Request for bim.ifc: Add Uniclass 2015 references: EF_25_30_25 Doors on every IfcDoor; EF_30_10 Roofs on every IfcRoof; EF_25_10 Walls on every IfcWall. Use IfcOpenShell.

First a look at what the model holds.

```python
import ifcopenshell

model = ifcopenshell.open("bim.ifc")
print(model.schema)
print("classifications:", [c.Name for c in model.by_type("IfcClassification")])
for ifc_class in ("IfcDoor", "IfcRoof", "IfcStair", "IfcWall", "IfcWindow"):
    print(ifc_class, len(model.by_type(ifc_class)))
```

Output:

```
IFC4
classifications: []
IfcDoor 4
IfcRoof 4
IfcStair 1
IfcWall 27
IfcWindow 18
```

```python
import ifcopenshell
import ifcopenshell.api.classification

model = ifcopenshell.open("bim.ifc")

system = ifcopenshell.api.classification.add_classification(model, classification="Uniclass 2015")

codes = {
    "IfcDoor": ("EF_25_30_25", "Doors"),
    "IfcRoof": ("EF_30_10", "Roofs"),
    "IfcWall": ("EF_25_10", "Walls"),
}
for ifc_class, (code, name) in codes.items():
    products = model.by_type(ifc_class)
    ifcopenshell.api.classification.add_reference(
        model, products=products, classification=system, identification=code, name=name
    )
    print(code, len(products))

model.write("bim_updated.ifc")
```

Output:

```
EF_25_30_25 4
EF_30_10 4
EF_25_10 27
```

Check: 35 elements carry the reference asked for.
